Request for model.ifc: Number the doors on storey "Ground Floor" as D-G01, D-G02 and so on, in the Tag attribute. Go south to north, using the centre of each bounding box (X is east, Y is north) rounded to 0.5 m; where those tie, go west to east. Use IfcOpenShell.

First a look at what the model holds.

```python
import ifcopenshell
import ifcopenshell.util.element
import ifcopenshell.util.placement

model = ifcopenshell.open("model.ifc")
print(model.schema)
storey = next(s for s in model.by_type("IfcBuildingStorey") if s.Name == "Ground Floor")
doors = [e for e in ifcopenshell.util.element.get_decomposition(storey) if e.is_a("IfcDoor")]
for e in sorted(doors, key=lambda e: e.id()):
    origin = ifcopenshell.util.placement.get_local_placement(e.ObjectPlacement)[:3, 3]
    print(e.id(), e.Tag, e.Name, origin.round(2) + 0.0, sep=" | ")
```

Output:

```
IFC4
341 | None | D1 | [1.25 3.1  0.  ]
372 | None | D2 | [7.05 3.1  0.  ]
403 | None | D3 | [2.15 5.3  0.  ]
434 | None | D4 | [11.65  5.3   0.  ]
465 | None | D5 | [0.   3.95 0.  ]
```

```python
import ifcopenshell
import ifcopenshell.geom
import ifcopenshell.util.element
import ifcopenshell.util.shape

model = ifcopenshell.open("model.ifc")
settings = ifcopenshell.geom.settings()
settings.set("use-world-coords", True)


def centre(element):
    shape = ifcopenshell.geom.create_shape(settings, element)
    return ifcopenshell.util.shape.get_bbox_centroid(shape.geometry)


storey = next(s for s in model.by_type("IfcBuildingStorey") if s.Name == "Ground Floor")
doors = [e for e in ifcopenshell.util.element.get_decomposition(storey) if e.is_a("IfcDoor")]

# Insertion points can sit at a corner or the storey origin, so sort by the geometry (in metres).
centres = {e: centre(e) for e in doors}
doors.sort(key=lambda e: (round(centres[e][1] / 0.5), centres[e][0]))

for i, e in enumerate(doors, start=1):
    number = f"D-G{i:02d}"
    e.Tag = number
    print(e.id(), number)

model.write("model-out.ifc")
```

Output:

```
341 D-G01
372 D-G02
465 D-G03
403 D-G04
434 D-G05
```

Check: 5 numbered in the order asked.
